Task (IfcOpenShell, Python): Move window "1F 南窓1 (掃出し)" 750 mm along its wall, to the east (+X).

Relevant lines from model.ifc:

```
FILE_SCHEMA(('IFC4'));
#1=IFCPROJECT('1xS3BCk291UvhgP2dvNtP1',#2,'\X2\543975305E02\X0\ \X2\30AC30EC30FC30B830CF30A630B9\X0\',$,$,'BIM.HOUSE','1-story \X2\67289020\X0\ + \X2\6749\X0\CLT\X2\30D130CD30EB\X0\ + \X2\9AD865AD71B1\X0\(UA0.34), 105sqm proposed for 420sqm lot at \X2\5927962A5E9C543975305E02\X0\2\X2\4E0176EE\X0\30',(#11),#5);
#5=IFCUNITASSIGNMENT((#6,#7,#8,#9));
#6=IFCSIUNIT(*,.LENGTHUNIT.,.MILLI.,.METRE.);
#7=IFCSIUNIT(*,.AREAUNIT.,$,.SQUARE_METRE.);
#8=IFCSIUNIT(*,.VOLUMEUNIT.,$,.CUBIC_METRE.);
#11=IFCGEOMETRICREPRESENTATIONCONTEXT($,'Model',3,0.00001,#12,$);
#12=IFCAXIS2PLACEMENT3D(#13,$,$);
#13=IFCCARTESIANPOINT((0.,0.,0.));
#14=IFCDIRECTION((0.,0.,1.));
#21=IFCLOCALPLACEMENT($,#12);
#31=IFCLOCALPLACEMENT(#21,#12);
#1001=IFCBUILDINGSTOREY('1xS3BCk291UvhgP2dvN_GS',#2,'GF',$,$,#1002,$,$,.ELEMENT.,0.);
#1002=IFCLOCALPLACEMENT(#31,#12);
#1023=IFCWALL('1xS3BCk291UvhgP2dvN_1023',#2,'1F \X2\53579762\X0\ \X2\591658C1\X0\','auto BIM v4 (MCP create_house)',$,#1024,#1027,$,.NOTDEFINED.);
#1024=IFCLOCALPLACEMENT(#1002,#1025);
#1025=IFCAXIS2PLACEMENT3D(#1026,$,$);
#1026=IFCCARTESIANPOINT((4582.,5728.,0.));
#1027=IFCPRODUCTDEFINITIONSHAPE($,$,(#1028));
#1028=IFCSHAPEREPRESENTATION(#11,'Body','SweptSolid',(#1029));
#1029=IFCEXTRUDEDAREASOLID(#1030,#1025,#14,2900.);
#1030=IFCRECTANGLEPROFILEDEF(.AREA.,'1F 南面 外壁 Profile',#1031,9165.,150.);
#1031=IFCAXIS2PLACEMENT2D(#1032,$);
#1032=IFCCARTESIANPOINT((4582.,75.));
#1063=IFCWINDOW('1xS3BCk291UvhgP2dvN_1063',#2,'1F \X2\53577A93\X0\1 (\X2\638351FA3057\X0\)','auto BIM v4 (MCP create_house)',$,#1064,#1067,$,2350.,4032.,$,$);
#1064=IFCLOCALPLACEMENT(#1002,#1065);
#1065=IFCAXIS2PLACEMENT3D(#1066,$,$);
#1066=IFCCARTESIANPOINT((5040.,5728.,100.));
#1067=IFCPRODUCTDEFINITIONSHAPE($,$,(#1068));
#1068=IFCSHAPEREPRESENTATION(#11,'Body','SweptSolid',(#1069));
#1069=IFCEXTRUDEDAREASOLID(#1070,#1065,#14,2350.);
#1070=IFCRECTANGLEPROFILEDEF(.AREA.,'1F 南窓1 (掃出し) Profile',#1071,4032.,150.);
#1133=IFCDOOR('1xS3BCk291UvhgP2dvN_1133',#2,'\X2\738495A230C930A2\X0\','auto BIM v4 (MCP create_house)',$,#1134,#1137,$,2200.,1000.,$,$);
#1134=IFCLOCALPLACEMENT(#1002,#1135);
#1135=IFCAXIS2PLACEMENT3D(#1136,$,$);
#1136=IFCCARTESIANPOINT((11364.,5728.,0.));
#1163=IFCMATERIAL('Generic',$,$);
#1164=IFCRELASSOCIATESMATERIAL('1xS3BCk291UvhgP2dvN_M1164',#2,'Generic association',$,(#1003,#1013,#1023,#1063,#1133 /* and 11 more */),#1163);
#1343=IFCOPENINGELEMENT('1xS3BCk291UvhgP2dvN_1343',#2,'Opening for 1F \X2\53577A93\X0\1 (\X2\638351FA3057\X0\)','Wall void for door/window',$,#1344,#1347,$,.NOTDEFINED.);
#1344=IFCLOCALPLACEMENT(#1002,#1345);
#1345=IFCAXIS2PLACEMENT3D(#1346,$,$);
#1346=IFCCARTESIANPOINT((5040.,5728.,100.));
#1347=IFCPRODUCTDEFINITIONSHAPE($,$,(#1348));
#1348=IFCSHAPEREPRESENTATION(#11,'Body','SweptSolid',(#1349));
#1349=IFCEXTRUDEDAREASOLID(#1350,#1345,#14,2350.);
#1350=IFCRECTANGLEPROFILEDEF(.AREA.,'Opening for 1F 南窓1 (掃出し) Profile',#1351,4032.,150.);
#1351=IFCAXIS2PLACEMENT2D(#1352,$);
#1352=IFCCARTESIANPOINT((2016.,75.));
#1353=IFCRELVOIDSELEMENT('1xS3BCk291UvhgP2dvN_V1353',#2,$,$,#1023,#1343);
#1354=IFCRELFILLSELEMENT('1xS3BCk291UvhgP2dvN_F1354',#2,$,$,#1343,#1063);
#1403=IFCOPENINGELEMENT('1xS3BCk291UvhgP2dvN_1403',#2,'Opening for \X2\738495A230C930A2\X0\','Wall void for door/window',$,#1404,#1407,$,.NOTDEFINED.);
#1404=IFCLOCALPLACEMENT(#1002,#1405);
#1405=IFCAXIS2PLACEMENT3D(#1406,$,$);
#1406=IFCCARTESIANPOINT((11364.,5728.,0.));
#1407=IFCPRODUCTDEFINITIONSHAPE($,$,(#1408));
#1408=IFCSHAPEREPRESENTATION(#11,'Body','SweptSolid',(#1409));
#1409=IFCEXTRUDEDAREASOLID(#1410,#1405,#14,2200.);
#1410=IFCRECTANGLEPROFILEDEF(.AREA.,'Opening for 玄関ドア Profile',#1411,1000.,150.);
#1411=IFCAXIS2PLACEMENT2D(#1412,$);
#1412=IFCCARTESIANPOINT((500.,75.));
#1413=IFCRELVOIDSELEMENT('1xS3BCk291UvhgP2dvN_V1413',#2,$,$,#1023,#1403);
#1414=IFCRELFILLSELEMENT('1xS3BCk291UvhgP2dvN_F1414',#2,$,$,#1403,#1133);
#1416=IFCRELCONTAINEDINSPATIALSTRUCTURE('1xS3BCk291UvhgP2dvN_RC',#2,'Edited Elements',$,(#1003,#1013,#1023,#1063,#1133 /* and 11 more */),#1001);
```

```python
import ifcopenshell
import ifcopenshell.api.geometry
import ifcopenshell.util.placement
import ifcopenshell.util.unit

model = ifcopenshell.open("model.ifc")
unit_scale = ifcopenshell.util.unit.calculate_unit_scale(model)

window = model.by_guid("1xS3BCk291UvhgP2dvN_1063")
opening = window.FillsVoids[0].RelatingOpeningElement
wall = opening.VoidsElements[0].RelatingBuildingElement

wall_matrix = ifcopenshell.util.placement.get_local_placement(wall.ObjectPlacement)
shift = wall_matrix[:3, 0] * 0.75 / unit_scale
before = ifcopenshell.util.placement.get_local_placement(window.ObjectPlacement)[:3, 3].copy()

# The window is not placed relative to its opening, so move both.
for product in (opening, window):
    matrix = ifcopenshell.util.placement.get_local_placement(product.ObjectPlacement)
    matrix[:3, 3] += shift
    ifcopenshell.api.geometry.edit_object_placement(model, product=product, matrix=matrix, is_si=False)

after = ifcopenshell.util.placement.get_local_placement(window.ObjectPlacement)[:3, 3]
print("window moved by", (after - before).round(3) + 0.0)

model.write("model_updated.ifc")
```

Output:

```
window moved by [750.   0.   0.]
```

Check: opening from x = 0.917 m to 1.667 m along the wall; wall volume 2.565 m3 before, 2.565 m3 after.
